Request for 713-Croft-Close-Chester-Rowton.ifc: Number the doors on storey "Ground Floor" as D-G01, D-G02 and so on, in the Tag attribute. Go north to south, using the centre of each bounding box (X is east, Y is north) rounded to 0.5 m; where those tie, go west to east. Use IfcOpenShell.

First a look at what the model holds.

```python
import ifcopenshell
import ifcopenshell.util.element
import ifcopenshell.util.placement

model = ifcopenshell.open("713-Croft-Close-Chester-Rowton.ifc")
print(model.schema)
storey = next(s for s in model.by_type("IfcBuildingStorey") if s.Name == "Ground Floor")
doors = [e for e in ifcopenshell.util.element.get_decomposition(storey) if e.is_a("IfcDoor")]
for e in sorted(doors, key=lambda e: e.id()):
    origin = ifcopenshell.util.placement.get_local_placement(e.ObjectPlacement)[:3, 3]
    print(e.id(), e.Tag, e.Name, origin.round(2) + 0.0, sep=" | ")
```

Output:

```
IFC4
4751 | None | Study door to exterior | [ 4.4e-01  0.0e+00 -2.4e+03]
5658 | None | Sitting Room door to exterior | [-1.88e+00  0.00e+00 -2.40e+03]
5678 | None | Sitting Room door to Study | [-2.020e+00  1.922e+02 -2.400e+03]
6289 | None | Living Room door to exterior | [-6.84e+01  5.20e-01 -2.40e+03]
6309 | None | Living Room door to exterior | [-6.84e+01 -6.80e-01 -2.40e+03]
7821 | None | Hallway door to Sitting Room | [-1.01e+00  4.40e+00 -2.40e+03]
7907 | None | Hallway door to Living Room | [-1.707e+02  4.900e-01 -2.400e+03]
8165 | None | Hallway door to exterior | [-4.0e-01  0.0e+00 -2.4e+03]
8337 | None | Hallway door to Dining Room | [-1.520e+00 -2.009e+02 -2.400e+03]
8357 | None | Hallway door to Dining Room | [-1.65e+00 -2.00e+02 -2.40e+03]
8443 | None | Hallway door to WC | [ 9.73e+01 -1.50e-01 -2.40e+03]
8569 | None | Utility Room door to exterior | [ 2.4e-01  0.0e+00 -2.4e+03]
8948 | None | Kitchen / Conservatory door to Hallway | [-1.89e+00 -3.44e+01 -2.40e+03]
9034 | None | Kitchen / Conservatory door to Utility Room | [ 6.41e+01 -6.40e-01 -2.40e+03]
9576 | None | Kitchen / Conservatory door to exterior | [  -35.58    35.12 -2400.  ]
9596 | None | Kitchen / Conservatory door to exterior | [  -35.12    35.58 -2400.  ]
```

```python
import ifcopenshell
import ifcopenshell.geom
import ifcopenshell.util.element
import ifcopenshell.util.shape

model = ifcopenshell.open("713-Croft-Close-Chester-Rowton.ifc")
settings = ifcopenshell.geom.settings()
settings.set("use-world-coords", True)


def centre(element):
    shape = ifcopenshell.geom.create_shape(settings, element)
    return ifcopenshell.util.shape.get_bbox_centroid(shape.geometry)


storey = next(s for s in model.by_type("IfcBuildingStorey") if s.Name == "Ground Floor")
doors = [e for e in ifcopenshell.util.element.get_decomposition(storey) if e.is_a("IfcDoor")]

# Insertion points can sit at a corner or the storey origin, so sort by the geometry (in metres).
centres = {e: centre(e) for e in doors}
doors.sort(key=lambda e: (-round(centres[e][1] / 0.5), centres[e][0]))

for i, e in enumerate(doors, start=1):
    number = f"D-G{i:02d}"
    e.Tag = number
    print(e.id(), number)

model.write("713-Croft-Close-Chester-Rowton_rev.ifc")
```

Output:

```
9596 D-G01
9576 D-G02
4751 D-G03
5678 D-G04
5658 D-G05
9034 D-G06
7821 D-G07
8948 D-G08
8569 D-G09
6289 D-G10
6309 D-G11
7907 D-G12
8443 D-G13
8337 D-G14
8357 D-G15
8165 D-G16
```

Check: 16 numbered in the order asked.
